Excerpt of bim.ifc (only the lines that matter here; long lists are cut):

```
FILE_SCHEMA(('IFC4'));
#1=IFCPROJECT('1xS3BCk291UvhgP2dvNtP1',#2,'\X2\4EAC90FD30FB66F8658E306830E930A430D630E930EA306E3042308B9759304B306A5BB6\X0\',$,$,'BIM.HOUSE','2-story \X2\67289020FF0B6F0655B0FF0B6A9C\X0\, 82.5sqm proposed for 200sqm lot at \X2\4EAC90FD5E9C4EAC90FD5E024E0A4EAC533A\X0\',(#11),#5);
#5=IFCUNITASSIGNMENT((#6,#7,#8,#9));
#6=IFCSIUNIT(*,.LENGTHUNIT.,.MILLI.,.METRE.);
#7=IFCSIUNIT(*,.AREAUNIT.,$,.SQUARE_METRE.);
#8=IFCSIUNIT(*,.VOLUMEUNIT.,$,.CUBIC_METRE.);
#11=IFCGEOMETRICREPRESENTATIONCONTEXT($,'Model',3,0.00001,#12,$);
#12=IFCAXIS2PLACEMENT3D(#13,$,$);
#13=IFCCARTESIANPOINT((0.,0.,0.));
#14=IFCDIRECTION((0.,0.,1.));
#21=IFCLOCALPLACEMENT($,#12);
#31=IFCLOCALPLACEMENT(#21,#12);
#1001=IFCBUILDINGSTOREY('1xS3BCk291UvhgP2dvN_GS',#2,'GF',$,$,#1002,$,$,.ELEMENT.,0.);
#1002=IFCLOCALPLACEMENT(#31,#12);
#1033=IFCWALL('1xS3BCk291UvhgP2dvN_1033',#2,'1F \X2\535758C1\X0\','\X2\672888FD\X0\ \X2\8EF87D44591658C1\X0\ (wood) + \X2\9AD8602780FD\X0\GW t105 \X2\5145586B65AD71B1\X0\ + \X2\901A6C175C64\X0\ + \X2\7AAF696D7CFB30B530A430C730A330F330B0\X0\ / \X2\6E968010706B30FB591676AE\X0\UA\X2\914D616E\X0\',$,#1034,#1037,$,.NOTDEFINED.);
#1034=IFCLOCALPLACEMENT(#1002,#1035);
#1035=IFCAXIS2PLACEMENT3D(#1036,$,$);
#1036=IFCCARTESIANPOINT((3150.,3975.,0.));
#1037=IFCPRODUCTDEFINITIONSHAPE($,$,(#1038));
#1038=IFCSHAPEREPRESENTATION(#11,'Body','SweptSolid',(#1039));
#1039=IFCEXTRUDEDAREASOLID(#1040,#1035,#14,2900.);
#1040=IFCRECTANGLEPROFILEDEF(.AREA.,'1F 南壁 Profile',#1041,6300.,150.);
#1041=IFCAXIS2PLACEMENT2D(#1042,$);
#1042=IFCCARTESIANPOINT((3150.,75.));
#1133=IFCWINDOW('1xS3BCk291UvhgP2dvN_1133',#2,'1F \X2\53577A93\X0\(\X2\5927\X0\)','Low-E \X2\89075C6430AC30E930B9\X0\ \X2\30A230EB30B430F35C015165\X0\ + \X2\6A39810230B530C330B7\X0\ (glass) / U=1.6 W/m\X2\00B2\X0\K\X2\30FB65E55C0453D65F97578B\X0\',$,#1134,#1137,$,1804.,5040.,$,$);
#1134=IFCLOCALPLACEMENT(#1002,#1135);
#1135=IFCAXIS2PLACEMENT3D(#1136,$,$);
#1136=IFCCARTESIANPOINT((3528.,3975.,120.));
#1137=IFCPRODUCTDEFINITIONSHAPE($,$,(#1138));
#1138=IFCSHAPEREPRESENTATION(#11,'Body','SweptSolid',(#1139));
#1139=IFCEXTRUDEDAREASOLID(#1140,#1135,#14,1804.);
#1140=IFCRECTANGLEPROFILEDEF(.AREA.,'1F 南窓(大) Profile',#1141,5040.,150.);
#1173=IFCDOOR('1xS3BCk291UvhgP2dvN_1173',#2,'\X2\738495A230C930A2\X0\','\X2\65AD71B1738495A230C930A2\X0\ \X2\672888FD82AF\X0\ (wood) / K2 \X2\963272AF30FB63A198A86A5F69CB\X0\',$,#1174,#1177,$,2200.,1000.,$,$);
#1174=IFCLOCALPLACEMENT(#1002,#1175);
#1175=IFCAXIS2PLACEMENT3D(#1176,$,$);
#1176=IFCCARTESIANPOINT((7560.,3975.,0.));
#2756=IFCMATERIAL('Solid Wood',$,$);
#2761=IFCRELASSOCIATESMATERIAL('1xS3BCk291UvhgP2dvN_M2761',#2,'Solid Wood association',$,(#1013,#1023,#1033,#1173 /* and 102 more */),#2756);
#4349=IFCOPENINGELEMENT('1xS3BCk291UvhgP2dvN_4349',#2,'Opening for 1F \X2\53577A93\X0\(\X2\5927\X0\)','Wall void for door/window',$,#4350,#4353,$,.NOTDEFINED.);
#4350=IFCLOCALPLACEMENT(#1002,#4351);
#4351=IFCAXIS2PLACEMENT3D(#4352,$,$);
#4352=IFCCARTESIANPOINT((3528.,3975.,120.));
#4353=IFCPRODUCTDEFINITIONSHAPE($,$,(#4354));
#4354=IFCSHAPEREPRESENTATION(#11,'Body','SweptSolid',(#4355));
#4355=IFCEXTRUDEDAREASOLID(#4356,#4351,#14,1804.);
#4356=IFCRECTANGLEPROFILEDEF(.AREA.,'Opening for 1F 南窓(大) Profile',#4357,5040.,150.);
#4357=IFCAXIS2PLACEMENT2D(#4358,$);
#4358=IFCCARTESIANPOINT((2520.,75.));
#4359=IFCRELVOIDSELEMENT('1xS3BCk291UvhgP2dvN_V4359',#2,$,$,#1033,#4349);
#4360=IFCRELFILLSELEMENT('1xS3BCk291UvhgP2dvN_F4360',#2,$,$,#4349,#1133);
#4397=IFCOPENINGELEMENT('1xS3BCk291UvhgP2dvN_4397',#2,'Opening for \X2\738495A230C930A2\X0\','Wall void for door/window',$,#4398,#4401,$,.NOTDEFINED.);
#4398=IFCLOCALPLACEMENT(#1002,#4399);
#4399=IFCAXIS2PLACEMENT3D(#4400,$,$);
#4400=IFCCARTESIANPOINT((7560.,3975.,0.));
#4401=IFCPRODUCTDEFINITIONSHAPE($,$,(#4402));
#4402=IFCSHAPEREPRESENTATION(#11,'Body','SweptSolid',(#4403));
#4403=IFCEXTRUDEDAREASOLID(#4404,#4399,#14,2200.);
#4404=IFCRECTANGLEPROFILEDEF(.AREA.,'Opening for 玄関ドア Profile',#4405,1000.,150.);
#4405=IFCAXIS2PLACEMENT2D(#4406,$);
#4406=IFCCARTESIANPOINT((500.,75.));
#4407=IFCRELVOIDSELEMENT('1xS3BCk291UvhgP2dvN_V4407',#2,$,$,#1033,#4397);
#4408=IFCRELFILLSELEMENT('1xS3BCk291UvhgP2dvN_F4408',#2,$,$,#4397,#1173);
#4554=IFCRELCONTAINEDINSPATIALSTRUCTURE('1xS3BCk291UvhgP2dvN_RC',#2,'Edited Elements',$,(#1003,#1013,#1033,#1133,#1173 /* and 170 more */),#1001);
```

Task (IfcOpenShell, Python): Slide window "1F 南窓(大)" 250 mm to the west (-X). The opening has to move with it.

```python
import ifcopenshell
import ifcopenshell.api.geometry
import ifcopenshell.util.placement
import ifcopenshell.util.unit

model = ifcopenshell.open("bim.ifc")
unit_scale = ifcopenshell.util.unit.calculate_unit_scale(model)

window = model.by_guid("1xS3BCk291UvhgP2dvN_1133")
opening = window.FillsVoids[0].RelatingOpeningElement
wall = opening.VoidsElements[0].RelatingBuildingElement

wall_matrix = ifcopenshell.util.placement.get_local_placement(wall.ObjectPlacement)
shift = wall_matrix[:3, 0] * -0.25 / unit_scale
before = ifcopenshell.util.placement.get_local_placement(window.ObjectPlacement)[:3, 3].copy()

# The window is not placed relative to its opening, so move both.
for product in (opening, window):
    matrix = ifcopenshell.util.placement.get_local_placement(product.ObjectPlacement)
    matrix[:3, 3] += shift
    ifcopenshell.api.geometry.edit_object_placement(model, product=product, matrix=matrix, is_si=False)

after = ifcopenshell.util.placement.get_local_placement(window.ObjectPlacement)[:3, 3]
print("window moved by", (after - before).round(3) + 0.0)

model.write("bim_updated.ifc")
```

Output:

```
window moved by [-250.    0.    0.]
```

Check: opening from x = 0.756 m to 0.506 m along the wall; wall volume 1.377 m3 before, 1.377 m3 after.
